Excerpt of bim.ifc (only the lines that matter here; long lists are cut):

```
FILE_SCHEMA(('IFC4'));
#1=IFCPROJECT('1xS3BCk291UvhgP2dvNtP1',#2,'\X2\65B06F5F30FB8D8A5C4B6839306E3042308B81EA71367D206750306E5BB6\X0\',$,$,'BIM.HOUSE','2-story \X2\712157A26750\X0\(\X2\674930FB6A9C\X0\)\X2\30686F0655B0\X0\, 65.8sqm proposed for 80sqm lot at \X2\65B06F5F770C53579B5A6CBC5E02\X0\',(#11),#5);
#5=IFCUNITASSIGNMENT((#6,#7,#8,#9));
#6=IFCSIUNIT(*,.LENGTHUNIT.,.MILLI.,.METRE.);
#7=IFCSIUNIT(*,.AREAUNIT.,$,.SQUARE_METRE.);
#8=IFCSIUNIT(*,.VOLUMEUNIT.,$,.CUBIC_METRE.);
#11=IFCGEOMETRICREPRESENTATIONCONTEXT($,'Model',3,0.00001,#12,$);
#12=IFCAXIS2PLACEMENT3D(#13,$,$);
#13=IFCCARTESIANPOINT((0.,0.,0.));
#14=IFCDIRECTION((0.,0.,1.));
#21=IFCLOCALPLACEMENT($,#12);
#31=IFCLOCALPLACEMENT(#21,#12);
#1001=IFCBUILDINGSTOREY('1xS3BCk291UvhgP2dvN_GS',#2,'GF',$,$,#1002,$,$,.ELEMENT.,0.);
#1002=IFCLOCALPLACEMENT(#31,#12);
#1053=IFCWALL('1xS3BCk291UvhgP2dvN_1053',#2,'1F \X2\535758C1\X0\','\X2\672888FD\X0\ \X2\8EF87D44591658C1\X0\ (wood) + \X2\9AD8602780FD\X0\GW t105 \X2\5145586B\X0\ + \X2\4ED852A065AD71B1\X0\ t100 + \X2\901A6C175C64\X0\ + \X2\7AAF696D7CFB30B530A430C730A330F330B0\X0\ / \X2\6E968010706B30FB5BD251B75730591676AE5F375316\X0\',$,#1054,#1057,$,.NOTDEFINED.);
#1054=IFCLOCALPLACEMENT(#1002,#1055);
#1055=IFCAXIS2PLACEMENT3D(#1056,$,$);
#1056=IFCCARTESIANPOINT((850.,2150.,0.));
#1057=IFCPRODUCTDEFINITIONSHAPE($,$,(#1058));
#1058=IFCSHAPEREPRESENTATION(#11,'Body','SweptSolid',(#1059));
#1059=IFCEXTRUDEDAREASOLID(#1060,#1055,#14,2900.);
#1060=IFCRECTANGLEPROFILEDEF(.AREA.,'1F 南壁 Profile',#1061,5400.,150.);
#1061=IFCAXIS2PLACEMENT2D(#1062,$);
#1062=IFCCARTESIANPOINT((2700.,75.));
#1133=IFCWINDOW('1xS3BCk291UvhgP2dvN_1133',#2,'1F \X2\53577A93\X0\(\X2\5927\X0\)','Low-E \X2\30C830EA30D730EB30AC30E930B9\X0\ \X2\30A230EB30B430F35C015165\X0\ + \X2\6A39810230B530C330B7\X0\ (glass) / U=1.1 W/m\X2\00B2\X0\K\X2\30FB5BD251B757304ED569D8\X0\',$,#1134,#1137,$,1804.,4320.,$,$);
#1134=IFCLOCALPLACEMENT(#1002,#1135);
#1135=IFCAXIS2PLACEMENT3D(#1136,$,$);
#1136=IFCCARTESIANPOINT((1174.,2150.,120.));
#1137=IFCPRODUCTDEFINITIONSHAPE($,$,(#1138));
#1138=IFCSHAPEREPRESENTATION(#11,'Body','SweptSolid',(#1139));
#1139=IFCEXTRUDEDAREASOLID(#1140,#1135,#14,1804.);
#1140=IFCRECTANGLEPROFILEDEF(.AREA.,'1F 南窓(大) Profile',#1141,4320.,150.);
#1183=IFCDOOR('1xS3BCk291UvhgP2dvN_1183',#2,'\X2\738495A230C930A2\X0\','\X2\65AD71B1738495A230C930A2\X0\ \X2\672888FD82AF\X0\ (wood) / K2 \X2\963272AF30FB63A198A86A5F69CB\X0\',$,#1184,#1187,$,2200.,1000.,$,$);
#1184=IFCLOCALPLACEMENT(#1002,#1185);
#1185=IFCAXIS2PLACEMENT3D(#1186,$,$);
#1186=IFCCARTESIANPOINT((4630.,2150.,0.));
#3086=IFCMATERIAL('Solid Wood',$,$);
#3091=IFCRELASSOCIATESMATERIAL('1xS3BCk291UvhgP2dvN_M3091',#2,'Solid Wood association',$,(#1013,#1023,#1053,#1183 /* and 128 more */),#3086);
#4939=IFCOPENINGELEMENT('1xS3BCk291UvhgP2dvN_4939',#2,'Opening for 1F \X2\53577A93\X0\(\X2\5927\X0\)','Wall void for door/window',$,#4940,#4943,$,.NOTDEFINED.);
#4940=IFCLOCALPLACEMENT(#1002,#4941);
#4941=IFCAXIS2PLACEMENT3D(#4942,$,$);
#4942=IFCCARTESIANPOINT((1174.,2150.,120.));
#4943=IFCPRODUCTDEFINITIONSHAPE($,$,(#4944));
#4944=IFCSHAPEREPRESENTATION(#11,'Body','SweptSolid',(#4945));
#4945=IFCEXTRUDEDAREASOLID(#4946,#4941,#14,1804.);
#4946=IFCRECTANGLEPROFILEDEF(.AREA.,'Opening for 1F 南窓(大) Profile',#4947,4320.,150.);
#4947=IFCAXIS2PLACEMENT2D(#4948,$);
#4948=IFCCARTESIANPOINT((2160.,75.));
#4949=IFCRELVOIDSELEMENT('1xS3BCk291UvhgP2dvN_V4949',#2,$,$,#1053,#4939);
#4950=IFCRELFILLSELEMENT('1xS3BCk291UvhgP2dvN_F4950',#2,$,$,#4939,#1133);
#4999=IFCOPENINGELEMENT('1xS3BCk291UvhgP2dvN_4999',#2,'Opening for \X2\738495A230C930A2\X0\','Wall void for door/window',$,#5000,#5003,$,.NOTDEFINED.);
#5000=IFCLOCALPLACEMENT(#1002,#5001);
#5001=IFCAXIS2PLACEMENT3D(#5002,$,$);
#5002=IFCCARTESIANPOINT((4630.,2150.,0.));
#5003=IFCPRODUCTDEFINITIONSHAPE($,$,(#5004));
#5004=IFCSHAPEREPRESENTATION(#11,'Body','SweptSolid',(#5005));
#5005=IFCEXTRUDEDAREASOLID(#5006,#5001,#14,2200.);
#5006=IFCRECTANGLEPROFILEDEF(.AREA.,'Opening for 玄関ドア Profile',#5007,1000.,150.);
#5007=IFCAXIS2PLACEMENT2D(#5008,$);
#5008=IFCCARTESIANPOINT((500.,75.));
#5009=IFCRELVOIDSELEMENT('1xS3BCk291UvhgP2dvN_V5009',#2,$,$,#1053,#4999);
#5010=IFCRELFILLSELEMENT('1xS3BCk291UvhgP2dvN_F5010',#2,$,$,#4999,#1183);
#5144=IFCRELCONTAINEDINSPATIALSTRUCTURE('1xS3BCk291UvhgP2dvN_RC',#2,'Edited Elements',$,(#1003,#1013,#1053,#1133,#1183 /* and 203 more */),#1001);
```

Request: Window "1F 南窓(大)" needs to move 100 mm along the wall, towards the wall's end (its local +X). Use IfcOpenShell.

```python
import ifcopenshell
import ifcopenshell.api.geometry
import ifcopenshell.util.placement
import ifcopenshell.util.unit

model = ifcopenshell.open("bim.ifc")
unit_scale = ifcopenshell.util.unit.calculate_unit_scale(model)

window = model.by_guid("1xS3BCk291UvhgP2dvN_1133")
opening = window.FillsVoids[0].RelatingOpeningElement
wall = opening.VoidsElements[0].RelatingBuildingElement

wall_matrix = ifcopenshell.util.placement.get_local_placement(wall.ObjectPlacement)
shift = wall_matrix[:3, 0] * 0.1 / unit_scale
before = ifcopenshell.util.placement.get_local_placement(window.ObjectPlacement)[:3, 3].copy()

# The window is not placed relative to its opening, so move both.
for product in (opening, window):
    matrix = ifcopenshell.util.placement.get_local_placement(product.ObjectPlacement)
    matrix[:3, 3] += shift
    ifcopenshell.api.geometry.edit_object_placement(model, product=product, matrix=matrix, is_si=False)

after = ifcopenshell.util.placement.get_local_placement(window.ObjectPlacement)[:3, 3]
print("window moved by", (after - before).round(3) + 0.0)

model.write("bim_edited.ifc")
```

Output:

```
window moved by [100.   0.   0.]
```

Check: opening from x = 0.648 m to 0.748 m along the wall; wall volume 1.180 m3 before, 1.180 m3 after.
